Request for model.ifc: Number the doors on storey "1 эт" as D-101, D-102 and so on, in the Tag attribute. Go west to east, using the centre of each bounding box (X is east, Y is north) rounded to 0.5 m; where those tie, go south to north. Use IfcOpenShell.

First a look at what the model holds.

```python
import ifcopenshell
import ifcopenshell.util.element
import ifcopenshell.util.placement

model = ifcopenshell.open("model.ifc")
print(model.schema)
storey = next(s for s in model.by_type("IfcBuildingStorey") if s.Name == "1 эт")
doors = [e for e in ifcopenshell.util.element.get_decomposition(storey) if e.is_a("IfcDoor")]
for e in sorted(doors, key=lambda e: e.id()):
    origin = ifcopenshell.util.placement.get_local_placement(e.ObjectPlacement)[:3, 3]
    print(e.id(), e.Tag, e.Name, origin.round(2) + 0.0, sep=" | ")
```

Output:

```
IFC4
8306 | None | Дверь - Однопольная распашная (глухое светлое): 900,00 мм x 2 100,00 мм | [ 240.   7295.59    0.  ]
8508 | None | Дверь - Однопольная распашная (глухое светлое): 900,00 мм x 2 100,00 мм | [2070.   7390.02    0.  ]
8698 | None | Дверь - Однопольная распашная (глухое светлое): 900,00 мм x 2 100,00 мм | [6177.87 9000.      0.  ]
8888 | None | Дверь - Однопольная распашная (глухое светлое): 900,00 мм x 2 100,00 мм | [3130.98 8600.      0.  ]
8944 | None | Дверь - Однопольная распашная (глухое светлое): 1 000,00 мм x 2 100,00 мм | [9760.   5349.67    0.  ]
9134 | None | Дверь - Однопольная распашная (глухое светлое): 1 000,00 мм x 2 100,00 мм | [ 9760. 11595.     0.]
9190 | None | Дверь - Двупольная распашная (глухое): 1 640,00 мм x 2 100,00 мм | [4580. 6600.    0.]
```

```python
import ifcopenshell
import ifcopenshell.geom
import ifcopenshell.util.element
import ifcopenshell.util.shape

model = ifcopenshell.open("model.ifc")
settings = ifcopenshell.geom.settings()
settings.set("use-world-coords", True)


def centre(element):
    shape = ifcopenshell.geom.create_shape(settings, element)
    return ifcopenshell.util.shape.get_bbox_centroid(shape.geometry)


storey = next(s for s in model.by_type("IfcBuildingStorey") if s.Name == "1 эт")
doors = [e for e in ifcopenshell.util.element.get_decomposition(storey) if e.is_a("IfcDoor")]

# Insertion points can sit at a corner or the storey origin, so sort by the geometry (in metres).
centres = {e: centre(e) for e in doors}
doors.sort(key=lambda e: (round(centres[e][0] / 0.5), centres[e][1]))

for i, e in enumerate(doors, start=1):
    number = f"D-1{i:02d}"
    e.Tag = number
    print(e.id(), number)

model.write("model_edited.ifc")
```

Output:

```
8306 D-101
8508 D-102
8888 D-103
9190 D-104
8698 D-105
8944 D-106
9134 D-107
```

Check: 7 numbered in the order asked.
